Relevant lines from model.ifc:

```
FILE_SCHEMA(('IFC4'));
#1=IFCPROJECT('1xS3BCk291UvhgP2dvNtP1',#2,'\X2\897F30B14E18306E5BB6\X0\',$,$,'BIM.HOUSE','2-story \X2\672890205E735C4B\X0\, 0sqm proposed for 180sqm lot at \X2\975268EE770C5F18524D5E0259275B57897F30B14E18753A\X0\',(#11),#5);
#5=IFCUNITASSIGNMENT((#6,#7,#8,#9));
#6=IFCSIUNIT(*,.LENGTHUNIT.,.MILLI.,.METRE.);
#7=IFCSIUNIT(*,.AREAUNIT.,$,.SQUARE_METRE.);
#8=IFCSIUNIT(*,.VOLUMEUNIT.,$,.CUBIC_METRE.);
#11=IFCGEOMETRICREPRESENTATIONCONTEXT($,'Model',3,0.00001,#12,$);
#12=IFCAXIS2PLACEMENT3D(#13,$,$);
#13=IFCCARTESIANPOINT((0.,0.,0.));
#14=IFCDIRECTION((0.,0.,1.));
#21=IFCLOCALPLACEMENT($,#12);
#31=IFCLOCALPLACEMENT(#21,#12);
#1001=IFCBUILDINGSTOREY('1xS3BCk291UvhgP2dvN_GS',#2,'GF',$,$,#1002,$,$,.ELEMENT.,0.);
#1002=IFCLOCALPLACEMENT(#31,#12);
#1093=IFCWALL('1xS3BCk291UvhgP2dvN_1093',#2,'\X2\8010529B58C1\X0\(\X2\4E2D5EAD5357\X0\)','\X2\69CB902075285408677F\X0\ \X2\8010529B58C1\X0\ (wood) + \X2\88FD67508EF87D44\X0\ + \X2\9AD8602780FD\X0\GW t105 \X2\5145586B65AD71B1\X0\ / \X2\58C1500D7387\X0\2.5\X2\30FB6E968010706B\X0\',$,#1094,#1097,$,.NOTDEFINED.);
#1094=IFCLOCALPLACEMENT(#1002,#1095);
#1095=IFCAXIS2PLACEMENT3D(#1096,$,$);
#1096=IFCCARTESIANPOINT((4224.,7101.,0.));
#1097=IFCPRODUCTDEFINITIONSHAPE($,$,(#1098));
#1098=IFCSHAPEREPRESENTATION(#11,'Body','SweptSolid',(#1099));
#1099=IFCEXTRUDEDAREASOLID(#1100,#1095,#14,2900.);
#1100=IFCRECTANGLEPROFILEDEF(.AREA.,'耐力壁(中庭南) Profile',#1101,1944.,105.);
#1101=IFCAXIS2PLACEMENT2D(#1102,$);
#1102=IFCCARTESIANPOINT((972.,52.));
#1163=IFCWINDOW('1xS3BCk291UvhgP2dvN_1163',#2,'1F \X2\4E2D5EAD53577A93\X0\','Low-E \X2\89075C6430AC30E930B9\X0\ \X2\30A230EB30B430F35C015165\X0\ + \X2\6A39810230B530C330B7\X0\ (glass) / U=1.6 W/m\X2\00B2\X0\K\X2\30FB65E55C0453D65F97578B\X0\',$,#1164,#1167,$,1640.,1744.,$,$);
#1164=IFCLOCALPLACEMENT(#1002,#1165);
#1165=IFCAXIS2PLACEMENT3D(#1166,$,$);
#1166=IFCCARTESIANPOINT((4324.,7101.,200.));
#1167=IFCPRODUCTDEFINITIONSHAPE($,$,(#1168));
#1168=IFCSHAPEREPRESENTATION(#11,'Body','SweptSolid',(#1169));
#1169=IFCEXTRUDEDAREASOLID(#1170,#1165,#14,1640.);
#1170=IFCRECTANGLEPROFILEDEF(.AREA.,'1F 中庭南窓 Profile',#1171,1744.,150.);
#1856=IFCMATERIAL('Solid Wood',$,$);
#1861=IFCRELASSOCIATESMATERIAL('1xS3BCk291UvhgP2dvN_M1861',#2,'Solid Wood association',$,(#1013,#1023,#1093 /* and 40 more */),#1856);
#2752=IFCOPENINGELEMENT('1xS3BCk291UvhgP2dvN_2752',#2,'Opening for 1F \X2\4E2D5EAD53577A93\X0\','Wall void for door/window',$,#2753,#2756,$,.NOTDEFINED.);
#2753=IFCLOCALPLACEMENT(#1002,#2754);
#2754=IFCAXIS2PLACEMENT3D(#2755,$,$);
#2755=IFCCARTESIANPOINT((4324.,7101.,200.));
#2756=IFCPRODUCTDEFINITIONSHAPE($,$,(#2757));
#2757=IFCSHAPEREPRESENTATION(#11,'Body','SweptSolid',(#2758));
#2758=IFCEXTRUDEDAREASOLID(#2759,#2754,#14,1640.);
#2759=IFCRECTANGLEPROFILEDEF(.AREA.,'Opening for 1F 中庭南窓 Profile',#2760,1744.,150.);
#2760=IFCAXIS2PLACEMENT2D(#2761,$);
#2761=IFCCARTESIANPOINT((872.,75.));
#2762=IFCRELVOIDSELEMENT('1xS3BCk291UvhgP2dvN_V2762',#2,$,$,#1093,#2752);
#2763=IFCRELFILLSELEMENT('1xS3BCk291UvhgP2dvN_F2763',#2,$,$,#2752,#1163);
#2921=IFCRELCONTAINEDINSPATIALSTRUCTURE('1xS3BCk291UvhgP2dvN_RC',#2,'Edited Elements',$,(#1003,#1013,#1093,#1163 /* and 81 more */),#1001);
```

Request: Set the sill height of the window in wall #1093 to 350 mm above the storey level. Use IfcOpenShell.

```python
import numpy as np
import ifcopenshell
import ifcopenshell.api.geometry
import ifcopenshell.geom
import ifcopenshell.util.element
import ifcopenshell.util.placement
import ifcopenshell.util.shape
import ifcopenshell.util.unit

model = ifcopenshell.open("model.ifc")
unit_scale = ifcopenshell.util.unit.calculate_unit_scale(model)

window = model.by_guid("1xS3BCk291UvhgP2dvN_1163")
opening = window.FillsVoids[0].RelatingOpeningElement
storey = ifcopenshell.util.element.get_container(window, ifc_class="IfcBuildingStorey")
level = ifcopenshell.util.placement.get_local_placement(storey.ObjectPlacement)[2, 3]

# The opening's origin need not be at the sill, so measure its lowest point.
shape = ifcopenshell.geom.create_shape(ifcopenshell.geom.settings(), opening)
bottom = ifcopenshell.util.shape.get_shape_bottom_elevation(shape, shape.geometry) / unit_scale
dz = level + 350.0 - bottom

shift = np.array([0.0, 0.0, dz])
# The window is not placed relative to its opening, so move both.
for product in (opening, window):
    matrix = ifcopenshell.util.placement.get_local_placement(product.ObjectPlacement)
    matrix[:3, 3] += shift
    ifcopenshell.api.geometry.edit_object_placement(model, product=product, matrix=matrix, is_si=False)

print(f"moved by {dz * unit_scale:+.3f} m")

model.write("model_updated.ifc")
```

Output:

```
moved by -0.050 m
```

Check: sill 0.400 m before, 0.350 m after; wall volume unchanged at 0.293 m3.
